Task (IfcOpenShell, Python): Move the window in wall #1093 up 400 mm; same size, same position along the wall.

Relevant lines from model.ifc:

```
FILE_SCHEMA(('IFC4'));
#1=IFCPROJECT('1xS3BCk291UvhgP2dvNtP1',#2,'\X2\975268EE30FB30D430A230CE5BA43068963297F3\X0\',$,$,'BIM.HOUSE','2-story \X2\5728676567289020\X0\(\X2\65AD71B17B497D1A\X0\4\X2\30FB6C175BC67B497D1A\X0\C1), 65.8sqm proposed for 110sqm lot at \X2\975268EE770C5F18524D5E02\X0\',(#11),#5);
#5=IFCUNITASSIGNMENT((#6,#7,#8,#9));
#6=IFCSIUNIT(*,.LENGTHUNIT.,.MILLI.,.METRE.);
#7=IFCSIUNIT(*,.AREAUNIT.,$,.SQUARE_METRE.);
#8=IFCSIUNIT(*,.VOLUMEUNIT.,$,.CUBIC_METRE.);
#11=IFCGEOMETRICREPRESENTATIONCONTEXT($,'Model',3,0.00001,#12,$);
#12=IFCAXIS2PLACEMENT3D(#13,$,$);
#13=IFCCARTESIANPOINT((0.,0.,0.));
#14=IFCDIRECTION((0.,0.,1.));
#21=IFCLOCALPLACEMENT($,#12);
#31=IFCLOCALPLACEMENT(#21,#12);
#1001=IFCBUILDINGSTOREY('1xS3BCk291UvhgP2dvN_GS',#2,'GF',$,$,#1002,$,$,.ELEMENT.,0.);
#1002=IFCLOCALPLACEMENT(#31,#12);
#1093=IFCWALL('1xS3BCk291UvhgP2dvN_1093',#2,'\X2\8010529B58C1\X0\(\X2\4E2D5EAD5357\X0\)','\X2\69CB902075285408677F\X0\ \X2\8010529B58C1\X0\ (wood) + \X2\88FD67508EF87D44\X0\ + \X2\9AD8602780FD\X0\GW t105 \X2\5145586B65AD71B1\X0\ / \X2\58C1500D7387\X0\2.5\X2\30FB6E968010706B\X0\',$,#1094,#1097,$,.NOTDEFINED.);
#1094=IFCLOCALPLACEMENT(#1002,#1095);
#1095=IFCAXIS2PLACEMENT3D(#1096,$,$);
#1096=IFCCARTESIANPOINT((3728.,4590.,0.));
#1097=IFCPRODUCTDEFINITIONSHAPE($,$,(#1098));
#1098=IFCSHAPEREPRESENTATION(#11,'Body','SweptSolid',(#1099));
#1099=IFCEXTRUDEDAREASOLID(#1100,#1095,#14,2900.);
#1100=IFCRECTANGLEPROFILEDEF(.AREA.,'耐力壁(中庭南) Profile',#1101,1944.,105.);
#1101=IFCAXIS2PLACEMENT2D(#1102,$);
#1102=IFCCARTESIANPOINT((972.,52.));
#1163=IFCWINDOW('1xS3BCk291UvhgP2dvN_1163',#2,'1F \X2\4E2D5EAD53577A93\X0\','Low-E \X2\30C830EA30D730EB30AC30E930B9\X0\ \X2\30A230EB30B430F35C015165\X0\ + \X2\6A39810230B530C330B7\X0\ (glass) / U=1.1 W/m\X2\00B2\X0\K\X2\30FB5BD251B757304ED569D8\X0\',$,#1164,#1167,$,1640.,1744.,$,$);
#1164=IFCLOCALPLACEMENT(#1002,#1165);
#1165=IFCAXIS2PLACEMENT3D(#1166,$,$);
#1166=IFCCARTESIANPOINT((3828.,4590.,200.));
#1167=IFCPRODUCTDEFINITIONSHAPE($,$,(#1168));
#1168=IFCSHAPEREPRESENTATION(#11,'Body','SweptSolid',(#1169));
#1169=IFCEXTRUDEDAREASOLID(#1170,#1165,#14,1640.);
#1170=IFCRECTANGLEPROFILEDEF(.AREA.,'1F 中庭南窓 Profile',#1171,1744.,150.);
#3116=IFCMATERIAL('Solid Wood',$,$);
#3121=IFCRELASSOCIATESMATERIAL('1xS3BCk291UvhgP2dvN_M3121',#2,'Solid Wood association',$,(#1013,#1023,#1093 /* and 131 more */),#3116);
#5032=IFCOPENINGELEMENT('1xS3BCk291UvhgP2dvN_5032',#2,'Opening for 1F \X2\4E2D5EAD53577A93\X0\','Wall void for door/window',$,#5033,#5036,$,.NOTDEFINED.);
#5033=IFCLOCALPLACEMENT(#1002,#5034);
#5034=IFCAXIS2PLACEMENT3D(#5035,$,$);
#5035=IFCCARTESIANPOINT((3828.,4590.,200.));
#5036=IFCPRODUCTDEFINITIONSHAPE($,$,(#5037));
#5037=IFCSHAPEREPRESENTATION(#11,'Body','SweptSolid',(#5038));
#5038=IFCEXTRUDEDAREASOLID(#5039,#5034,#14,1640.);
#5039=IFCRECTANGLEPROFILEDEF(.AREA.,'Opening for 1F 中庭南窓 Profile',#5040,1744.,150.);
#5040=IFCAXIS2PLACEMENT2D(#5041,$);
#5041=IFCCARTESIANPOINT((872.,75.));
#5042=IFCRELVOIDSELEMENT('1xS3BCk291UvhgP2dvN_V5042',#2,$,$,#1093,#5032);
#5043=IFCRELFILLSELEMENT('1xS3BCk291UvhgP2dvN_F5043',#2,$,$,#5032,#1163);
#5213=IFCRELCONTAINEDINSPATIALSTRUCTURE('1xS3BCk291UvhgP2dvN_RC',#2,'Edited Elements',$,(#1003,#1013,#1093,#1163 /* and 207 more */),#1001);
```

```python
import numpy as np
import ifcopenshell
import ifcopenshell.api.geometry
import ifcopenshell.util.placement
import ifcopenshell.util.unit

model = ifcopenshell.open("model.ifc")
unit_scale = ifcopenshell.util.unit.calculate_unit_scale(model)

window = model.by_guid("1xS3BCk291UvhgP2dvN_1163")
opening = window.FillsVoids[0].RelatingOpeningElement
dz = 0.4 / unit_scale

shift = np.array([0.0, 0.0, dz])
# The window is not placed relative to its opening, so move both.
for product in (opening, window):
    matrix = ifcopenshell.util.placement.get_local_placement(product.ObjectPlacement)
    matrix[:3, 3] += shift
    ifcopenshell.api.geometry.edit_object_placement(model, product=product, matrix=matrix, is_si=False)

print(f"moved by {dz * unit_scale:+.3f} m")

model.write("model_edited.ifc")
```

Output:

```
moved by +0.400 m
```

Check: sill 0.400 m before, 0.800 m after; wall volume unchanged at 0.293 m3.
